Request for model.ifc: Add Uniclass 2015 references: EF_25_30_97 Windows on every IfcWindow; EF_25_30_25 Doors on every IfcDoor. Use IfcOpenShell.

First a look at what the model holds.

```python
import ifcopenshell

model = ifcopenshell.open("model.ifc")
print(model.schema)
print("classifications:", [c.Name for c in model.by_type("IfcClassification")])
for ifc_class in ("IfcDoor", "IfcRoof", "IfcStair", "IfcWall", "IfcWindow"):
    print(ifc_class, len(model.by_type(ifc_class)))
```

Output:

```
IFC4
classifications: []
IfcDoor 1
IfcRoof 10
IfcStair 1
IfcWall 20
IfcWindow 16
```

```python
import ifcopenshell
import ifcopenshell.api.classification

model = ifcopenshell.open("model.ifc")

system = ifcopenshell.api.classification.add_classification(model, classification="Uniclass 2015")

codes = {
    "IfcWindow": ("EF_25_30_97", "Windows"),
    "IfcDoor": ("EF_25_30_25", "Doors"),
}
for ifc_class, (code, name) in codes.items():
    products = model.by_type(ifc_class)
    ifcopenshell.api.classification.add_reference(
        model, products=products, classification=system, identification=code, name=name
    )
    print(code, len(products))

model.write("model_rev.ifc")
```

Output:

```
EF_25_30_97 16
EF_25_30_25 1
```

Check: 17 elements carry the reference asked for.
